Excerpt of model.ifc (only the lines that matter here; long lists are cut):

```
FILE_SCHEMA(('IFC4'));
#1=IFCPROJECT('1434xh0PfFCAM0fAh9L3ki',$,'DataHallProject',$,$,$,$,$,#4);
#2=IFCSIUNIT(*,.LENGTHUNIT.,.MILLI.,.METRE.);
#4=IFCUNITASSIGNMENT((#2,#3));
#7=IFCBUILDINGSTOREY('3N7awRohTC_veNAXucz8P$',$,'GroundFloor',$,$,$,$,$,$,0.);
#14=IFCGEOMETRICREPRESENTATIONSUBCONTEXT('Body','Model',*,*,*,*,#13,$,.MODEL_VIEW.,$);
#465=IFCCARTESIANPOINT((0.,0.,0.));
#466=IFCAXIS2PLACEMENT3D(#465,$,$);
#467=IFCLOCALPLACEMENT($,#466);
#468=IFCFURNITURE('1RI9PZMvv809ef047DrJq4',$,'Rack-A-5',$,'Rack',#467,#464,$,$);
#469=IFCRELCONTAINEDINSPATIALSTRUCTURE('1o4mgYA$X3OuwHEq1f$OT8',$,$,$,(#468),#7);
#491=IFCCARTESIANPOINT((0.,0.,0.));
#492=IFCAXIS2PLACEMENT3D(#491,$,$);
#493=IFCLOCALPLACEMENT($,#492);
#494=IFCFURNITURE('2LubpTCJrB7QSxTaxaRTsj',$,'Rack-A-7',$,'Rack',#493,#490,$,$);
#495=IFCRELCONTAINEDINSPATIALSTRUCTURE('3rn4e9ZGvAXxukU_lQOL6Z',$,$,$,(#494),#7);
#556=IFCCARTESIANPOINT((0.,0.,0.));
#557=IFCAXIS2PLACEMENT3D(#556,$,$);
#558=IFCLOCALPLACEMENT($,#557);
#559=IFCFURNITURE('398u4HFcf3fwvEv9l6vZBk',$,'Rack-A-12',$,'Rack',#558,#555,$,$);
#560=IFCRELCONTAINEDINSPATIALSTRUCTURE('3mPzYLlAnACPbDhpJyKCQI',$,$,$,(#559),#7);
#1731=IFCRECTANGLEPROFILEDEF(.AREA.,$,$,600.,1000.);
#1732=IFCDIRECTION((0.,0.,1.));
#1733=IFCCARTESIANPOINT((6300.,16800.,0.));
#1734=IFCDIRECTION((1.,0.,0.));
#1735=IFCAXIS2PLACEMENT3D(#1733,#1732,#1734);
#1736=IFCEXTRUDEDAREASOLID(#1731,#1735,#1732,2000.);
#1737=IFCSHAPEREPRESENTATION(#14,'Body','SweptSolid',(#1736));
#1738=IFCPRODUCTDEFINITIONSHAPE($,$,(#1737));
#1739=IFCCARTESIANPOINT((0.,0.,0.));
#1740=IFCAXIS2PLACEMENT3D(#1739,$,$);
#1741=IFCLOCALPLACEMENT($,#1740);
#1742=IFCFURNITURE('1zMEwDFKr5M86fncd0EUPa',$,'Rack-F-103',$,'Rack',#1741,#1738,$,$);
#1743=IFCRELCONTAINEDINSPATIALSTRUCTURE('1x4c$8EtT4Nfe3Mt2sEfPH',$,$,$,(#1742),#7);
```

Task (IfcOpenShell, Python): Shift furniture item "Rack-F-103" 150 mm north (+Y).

```python
import ifcopenshell
import ifcopenshell.api.geometry
import ifcopenshell.util.placement
import ifcopenshell.util.unit

model = ifcopenshell.open("model.ifc")
unit_scale = ifcopenshell.util.unit.calculate_unit_scale(model)

item = model.by_guid("1zMEwDFKr5M86fncd0EUPa")
matrix = ifcopenshell.util.placement.get_local_placement(item.ObjectPlacement)
matrix[1, 3] += 0.15 / unit_scale
ifcopenshell.api.geometry.edit_object_placement(model, product=item, matrix=matrix, is_si=False)

print(ifcopenshell.util.placement.get_local_placement(item.ObjectPlacement).round(3) + 0.0)

model.write("model_rev.ifc")
```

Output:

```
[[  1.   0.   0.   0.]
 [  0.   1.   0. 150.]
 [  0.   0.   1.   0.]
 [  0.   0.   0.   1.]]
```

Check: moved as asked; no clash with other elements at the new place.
